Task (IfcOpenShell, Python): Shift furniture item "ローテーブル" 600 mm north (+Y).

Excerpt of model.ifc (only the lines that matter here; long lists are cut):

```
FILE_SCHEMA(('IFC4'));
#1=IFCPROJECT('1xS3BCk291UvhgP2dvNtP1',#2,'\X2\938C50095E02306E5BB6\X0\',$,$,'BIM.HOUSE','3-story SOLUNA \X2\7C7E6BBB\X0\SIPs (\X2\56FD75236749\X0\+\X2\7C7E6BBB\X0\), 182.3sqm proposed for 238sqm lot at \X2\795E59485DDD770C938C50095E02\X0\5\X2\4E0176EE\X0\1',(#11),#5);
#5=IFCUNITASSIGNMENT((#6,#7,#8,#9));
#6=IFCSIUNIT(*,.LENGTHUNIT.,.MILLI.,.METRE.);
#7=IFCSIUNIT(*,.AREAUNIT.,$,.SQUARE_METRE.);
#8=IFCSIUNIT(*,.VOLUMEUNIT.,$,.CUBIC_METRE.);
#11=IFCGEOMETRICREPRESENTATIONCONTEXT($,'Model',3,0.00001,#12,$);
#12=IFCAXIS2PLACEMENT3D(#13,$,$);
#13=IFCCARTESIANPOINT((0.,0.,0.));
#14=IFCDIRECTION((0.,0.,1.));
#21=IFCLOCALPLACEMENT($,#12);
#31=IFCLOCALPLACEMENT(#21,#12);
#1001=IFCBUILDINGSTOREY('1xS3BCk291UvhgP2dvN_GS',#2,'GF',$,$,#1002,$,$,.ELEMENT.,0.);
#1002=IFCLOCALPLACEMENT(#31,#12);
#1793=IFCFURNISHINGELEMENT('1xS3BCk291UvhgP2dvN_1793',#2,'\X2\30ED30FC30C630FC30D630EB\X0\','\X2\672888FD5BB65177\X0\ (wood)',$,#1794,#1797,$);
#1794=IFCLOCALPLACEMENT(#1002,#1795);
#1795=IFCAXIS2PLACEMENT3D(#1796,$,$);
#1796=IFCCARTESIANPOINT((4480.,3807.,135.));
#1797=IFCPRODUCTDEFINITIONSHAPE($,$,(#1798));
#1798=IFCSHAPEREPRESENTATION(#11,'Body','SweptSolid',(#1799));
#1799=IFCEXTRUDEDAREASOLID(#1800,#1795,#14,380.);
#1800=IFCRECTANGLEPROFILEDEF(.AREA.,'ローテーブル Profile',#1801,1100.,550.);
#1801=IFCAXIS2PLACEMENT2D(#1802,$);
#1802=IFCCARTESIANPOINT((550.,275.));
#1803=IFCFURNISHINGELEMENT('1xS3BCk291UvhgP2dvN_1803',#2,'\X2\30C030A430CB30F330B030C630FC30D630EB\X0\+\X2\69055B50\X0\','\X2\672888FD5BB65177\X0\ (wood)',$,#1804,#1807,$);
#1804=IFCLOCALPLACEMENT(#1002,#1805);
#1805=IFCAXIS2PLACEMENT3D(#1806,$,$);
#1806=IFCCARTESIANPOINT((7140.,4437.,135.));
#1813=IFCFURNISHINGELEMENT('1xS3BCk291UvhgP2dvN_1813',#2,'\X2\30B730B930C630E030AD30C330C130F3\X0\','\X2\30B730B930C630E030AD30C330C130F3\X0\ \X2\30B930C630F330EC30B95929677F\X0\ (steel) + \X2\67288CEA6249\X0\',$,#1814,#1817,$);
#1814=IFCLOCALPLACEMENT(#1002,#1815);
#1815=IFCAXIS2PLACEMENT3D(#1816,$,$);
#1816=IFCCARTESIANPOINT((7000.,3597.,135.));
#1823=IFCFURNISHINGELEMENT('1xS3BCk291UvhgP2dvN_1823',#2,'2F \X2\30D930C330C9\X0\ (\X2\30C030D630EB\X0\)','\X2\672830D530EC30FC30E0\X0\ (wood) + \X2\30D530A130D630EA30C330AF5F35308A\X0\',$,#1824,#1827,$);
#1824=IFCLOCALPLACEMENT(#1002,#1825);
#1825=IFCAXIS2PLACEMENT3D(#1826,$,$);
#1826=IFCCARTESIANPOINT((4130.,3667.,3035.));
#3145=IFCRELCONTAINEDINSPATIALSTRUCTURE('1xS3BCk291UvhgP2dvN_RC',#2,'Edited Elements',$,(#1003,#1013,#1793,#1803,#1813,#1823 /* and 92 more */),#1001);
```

```python
import ifcopenshell
import ifcopenshell.api.geometry
import ifcopenshell.util.placement
import ifcopenshell.util.unit

model = ifcopenshell.open("model.ifc")
unit_scale = ifcopenshell.util.unit.calculate_unit_scale(model)

item = model.by_id(1793)
matrix = ifcopenshell.util.placement.get_local_placement(item.ObjectPlacement)
matrix[1, 3] += 0.6 / unit_scale
ifcopenshell.api.geometry.edit_object_placement(model, product=item, matrix=matrix, is_si=False)

print(ifcopenshell.util.placement.get_local_placement(item.ObjectPlacement).round(3) + 0.0)

model.write("model_updated.ifc")
```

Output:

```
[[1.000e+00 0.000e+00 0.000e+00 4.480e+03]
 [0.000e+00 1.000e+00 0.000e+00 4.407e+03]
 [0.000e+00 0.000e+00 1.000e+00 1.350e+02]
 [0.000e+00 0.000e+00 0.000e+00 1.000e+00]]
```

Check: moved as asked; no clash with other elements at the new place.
